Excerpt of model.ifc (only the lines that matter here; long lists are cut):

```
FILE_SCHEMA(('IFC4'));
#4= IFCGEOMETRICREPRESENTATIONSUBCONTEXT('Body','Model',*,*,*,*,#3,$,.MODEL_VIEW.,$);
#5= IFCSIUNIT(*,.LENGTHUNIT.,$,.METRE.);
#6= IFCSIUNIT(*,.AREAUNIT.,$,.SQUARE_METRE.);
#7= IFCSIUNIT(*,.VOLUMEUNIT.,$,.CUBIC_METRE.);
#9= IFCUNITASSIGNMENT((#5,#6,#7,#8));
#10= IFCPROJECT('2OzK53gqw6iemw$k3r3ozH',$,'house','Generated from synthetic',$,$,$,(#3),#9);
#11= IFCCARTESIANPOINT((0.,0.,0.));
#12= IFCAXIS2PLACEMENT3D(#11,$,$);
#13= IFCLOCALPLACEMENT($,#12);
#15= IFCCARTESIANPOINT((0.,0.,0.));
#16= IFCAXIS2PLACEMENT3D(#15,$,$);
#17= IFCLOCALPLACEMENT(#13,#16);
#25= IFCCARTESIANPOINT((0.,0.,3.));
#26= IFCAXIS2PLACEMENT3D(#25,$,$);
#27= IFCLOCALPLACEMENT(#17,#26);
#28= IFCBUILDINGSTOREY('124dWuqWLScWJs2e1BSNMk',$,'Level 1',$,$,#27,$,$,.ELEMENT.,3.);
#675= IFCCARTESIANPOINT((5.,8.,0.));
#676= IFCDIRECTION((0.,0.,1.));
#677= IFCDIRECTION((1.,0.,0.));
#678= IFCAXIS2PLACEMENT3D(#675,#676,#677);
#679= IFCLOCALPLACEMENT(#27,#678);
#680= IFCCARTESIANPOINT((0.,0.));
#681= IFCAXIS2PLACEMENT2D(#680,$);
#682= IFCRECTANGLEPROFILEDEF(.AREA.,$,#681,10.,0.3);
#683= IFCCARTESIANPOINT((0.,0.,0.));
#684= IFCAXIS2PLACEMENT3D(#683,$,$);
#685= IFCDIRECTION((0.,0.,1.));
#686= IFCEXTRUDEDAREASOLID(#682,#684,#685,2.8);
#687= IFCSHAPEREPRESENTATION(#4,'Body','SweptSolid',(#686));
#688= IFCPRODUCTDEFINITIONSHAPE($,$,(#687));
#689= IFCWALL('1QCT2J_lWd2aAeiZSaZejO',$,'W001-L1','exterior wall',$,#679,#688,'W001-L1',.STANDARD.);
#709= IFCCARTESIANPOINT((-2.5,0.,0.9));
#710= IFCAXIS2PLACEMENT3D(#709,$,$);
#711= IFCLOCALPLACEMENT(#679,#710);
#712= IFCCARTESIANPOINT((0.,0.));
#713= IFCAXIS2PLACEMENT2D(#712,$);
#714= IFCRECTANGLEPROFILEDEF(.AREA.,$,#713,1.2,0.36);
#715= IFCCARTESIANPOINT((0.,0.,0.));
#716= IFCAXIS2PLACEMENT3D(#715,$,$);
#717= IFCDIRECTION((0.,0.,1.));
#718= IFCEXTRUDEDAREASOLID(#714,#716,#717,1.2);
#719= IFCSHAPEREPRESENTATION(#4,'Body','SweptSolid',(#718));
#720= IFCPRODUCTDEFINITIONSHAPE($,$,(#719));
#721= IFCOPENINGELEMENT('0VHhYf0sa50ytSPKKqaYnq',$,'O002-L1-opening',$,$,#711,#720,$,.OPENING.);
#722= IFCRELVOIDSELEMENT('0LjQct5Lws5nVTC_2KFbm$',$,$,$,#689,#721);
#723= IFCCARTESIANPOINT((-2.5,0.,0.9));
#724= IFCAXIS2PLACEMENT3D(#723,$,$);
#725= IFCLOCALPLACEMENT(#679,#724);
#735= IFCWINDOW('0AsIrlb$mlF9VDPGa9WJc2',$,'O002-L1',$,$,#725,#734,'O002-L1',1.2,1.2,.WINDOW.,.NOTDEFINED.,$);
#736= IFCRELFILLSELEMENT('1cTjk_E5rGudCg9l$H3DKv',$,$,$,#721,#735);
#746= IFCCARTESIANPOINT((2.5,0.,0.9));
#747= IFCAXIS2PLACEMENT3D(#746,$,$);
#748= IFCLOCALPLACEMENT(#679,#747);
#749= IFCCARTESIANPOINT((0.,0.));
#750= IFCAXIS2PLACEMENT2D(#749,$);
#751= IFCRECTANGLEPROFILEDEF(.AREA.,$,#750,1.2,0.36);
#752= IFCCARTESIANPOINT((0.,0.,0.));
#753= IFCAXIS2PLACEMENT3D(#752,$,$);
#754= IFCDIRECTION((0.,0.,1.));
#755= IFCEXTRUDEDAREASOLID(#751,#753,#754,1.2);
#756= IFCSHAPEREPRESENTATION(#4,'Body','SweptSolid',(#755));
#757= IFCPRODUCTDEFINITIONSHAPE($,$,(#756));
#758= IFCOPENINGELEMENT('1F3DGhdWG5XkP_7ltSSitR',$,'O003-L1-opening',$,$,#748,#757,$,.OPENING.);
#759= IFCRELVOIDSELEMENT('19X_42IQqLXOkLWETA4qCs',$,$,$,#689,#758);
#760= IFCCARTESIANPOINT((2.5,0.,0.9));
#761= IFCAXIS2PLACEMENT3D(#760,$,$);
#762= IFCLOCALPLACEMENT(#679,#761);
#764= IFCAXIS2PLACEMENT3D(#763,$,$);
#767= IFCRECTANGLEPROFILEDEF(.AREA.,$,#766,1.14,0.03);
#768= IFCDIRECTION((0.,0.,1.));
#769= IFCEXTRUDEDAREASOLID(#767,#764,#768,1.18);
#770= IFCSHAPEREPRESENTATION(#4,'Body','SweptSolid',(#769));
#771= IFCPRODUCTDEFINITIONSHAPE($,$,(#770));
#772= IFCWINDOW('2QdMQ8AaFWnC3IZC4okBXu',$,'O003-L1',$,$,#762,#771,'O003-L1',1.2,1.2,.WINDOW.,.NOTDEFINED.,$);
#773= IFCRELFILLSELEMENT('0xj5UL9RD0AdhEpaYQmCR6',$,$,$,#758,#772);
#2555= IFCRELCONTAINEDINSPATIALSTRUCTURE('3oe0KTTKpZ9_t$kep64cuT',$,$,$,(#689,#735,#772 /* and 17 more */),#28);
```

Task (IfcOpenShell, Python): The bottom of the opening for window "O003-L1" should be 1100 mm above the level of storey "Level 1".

```python
import numpy as np
import ifcopenshell
import ifcopenshell.api.geometry
import ifcopenshell.geom
import ifcopenshell.util.element
import ifcopenshell.util.placement
import ifcopenshell.util.shape
import ifcopenshell.util.unit

model = ifcopenshell.open("model.ifc")
unit_scale = ifcopenshell.util.unit.calculate_unit_scale(model)

window = model.by_guid("2QdMQ8AaFWnC3IZC4okBXu")
opening = window.FillsVoids[0].RelatingOpeningElement
storey = ifcopenshell.util.element.get_container(window, ifc_class="IfcBuildingStorey")
level = ifcopenshell.util.placement.get_local_placement(storey.ObjectPlacement)[2, 3]

# The opening's origin need not be at the sill, so measure its lowest point.
shape = ifcopenshell.geom.create_shape(ifcopenshell.geom.settings(), opening)
bottom = ifcopenshell.util.shape.get_shape_bottom_elevation(shape, shape.geometry) / unit_scale
dz = level + 1.1 - bottom

shift = np.array([0.0, 0.0, dz])
# The window is not placed relative to its opening, so move both.
for product in (opening, window):
    matrix = ifcopenshell.util.placement.get_local_placement(product.ObjectPlacement)
    matrix[:3, 3] += shift
    ifcopenshell.api.geometry.edit_object_placement(model, product=product, matrix=matrix, is_si=False)

print(f"moved by {dz * unit_scale:+.3f} m")

model.write("model_updated.ifc")
```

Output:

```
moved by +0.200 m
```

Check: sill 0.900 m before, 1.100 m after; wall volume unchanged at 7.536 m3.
